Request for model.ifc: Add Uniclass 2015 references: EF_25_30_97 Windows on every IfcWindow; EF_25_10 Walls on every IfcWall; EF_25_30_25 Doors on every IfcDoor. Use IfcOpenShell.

First a look at what the model holds.

```python
import ifcopenshell

model = ifcopenshell.open("model.ifc")
print(model.schema)
print("classifications:", [c.Name for c in model.by_type("IfcClassification")])
for ifc_class in ("IfcDoor", "IfcRoof", "IfcStair", "IfcWall", "IfcWindow"):
    print(ifc_class, len(model.by_type(ifc_class)))
```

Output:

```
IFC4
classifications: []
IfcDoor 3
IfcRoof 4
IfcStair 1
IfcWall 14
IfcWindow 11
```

```python
import ifcopenshell
import ifcopenshell.api.classification

model = ifcopenshell.open("model.ifc")

system = ifcopenshell.api.classification.add_classification(model, classification="Uniclass 2015")

codes = {
    "IfcWindow": ("EF_25_30_97", "Windows"),
    "IfcWall": ("EF_25_10", "Walls"),
    "IfcDoor": ("EF_25_30_25", "Doors"),
}
for ifc_class, (code, name) in codes.items():
    products = model.by_type(ifc_class)
    ifcopenshell.api.classification.add_reference(
        model, products=products, classification=system, identification=code, name=name
    )
    print(code, len(products))

model.write("model_rev.ifc")
```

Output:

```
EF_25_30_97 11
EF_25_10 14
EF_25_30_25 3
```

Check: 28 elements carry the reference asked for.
